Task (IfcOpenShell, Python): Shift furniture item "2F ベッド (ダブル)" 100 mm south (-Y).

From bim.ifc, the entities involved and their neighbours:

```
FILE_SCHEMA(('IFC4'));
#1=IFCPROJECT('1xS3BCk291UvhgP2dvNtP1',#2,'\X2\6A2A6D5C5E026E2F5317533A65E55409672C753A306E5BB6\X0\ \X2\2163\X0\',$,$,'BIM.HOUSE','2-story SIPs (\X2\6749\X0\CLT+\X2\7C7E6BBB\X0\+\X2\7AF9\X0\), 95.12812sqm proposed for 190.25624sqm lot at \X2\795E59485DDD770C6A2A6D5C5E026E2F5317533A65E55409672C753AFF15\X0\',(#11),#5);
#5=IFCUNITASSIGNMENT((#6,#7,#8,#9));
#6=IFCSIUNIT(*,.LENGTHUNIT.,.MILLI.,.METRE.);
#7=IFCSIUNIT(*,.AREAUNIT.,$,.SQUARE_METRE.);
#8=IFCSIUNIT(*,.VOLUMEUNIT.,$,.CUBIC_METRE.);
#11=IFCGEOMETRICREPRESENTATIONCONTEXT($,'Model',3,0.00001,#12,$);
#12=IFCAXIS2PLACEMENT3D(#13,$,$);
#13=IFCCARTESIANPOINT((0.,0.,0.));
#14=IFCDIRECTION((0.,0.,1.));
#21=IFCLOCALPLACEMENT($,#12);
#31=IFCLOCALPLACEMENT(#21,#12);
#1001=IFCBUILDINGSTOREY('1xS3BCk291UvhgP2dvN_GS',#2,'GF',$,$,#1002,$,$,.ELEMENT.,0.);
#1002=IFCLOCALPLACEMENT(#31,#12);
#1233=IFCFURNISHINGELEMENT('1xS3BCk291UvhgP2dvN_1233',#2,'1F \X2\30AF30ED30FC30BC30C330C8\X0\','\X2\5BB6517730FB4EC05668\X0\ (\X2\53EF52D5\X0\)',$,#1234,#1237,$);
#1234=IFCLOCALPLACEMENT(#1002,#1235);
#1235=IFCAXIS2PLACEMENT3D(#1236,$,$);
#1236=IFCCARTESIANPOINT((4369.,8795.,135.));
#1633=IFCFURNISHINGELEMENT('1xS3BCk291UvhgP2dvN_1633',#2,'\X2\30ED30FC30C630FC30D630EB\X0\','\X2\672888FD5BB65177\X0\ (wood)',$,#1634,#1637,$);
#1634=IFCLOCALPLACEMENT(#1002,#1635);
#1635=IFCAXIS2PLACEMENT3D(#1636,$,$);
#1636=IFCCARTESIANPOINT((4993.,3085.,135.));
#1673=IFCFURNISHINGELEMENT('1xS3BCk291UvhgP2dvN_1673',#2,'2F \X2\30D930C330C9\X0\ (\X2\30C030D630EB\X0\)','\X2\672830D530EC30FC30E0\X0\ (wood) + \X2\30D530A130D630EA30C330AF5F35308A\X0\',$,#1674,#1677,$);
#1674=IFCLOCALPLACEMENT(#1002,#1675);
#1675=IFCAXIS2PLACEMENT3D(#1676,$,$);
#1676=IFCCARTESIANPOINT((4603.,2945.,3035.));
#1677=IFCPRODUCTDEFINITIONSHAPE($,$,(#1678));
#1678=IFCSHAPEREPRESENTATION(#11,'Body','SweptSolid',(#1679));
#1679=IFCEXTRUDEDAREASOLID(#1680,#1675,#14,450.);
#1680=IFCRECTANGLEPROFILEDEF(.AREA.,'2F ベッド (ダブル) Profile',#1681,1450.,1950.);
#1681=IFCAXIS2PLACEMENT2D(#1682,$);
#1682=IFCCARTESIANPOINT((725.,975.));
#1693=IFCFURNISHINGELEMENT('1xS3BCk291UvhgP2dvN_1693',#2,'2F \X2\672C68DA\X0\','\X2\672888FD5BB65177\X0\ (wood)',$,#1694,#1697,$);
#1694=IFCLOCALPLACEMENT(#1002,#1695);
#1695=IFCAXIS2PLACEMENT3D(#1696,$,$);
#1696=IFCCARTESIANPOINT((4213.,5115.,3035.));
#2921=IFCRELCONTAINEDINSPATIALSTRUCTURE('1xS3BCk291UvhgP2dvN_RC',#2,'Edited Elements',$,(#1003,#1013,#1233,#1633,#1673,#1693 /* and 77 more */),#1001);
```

```python
import ifcopenshell
import ifcopenshell.api.geometry
import ifcopenshell.util.placement
import ifcopenshell.util.unit

model = ifcopenshell.open("bim.ifc")
unit_scale = ifcopenshell.util.unit.calculate_unit_scale(model)

item = model.by_id(1673)
matrix = ifcopenshell.util.placement.get_local_placement(item.ObjectPlacement)
matrix[1, 3] -= 0.1 / unit_scale
ifcopenshell.api.geometry.edit_object_placement(model, product=item, matrix=matrix, is_si=False)

print(ifcopenshell.util.placement.get_local_placement(item.ObjectPlacement).round(3) + 0.0)

model.write("bim_rev.ifc")
```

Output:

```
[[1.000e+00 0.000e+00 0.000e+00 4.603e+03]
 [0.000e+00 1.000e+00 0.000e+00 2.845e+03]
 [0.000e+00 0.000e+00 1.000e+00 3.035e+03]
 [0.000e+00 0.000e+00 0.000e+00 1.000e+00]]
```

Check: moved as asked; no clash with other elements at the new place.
